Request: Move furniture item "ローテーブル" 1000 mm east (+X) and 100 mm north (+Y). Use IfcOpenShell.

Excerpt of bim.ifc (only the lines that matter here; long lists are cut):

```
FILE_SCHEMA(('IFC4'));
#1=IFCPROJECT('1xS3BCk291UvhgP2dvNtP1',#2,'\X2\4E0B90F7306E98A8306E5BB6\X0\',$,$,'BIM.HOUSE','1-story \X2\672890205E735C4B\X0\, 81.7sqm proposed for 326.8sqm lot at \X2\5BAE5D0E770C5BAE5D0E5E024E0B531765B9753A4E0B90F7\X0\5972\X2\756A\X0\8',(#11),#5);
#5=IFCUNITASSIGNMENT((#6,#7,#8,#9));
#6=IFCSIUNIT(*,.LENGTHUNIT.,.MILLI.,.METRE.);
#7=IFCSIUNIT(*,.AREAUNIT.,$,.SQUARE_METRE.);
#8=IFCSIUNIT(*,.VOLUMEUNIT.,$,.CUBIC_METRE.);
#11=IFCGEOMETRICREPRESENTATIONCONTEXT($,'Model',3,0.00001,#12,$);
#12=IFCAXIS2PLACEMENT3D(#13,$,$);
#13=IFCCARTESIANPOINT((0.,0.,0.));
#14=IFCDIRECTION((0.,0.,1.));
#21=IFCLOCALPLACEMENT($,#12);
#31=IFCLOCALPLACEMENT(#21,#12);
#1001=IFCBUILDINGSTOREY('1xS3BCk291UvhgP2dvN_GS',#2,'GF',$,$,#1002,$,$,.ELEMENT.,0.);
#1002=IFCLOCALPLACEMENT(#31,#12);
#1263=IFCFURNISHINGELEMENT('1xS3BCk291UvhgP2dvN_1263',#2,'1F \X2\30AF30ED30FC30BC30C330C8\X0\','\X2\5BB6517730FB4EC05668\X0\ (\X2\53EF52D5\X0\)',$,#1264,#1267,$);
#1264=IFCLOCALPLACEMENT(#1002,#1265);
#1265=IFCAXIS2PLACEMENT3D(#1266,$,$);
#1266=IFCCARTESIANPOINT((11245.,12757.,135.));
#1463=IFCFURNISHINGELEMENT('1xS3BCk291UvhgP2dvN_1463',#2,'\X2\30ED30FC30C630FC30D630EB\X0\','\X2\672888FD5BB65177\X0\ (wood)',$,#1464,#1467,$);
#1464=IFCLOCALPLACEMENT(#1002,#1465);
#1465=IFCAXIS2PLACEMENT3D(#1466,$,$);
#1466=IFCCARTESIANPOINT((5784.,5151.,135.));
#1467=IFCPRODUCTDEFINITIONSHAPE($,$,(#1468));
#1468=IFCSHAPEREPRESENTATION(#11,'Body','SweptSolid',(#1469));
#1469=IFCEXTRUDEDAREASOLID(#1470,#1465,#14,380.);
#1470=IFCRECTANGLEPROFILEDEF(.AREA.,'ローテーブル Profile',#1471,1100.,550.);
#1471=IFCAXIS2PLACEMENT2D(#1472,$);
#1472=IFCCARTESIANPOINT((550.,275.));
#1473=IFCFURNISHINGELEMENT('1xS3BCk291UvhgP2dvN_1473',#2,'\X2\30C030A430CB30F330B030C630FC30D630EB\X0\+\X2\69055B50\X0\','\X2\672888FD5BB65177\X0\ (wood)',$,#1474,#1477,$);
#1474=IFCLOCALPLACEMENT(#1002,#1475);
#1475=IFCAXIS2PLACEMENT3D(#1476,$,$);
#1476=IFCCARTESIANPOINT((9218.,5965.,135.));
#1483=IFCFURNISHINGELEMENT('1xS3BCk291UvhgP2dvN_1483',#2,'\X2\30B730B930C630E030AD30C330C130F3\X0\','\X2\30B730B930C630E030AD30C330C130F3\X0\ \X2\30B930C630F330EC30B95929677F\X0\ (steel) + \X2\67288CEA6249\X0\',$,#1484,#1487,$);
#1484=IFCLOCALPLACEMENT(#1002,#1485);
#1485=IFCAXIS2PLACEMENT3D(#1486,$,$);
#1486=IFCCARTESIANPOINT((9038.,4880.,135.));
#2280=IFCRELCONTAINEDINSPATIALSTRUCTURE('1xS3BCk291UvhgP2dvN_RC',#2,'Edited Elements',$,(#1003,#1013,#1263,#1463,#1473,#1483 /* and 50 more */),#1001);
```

```python
import ifcopenshell
import ifcopenshell.api.geometry
import ifcopenshell.util.placement
import ifcopenshell.util.unit

model = ifcopenshell.open("bim.ifc")
unit_scale = ifcopenshell.util.unit.calculate_unit_scale(model)

item = model.by_guid("1xS3BCk291UvhgP2dvN_1463")
matrix = ifcopenshell.util.placement.get_local_placement(item.ObjectPlacement)
matrix[0, 3] += 1 / unit_scale
matrix[1, 3] += 0.1 / unit_scale
ifcopenshell.api.geometry.edit_object_placement(model, product=item, matrix=matrix, is_si=False)

print(ifcopenshell.util.placement.get_local_placement(item.ObjectPlacement).round(3) + 0.0)

model.write("bim_updated.ifc")
```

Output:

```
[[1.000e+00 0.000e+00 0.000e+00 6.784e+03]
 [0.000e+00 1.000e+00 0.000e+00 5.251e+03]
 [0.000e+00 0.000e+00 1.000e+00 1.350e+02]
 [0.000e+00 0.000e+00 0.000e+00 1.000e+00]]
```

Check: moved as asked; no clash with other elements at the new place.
